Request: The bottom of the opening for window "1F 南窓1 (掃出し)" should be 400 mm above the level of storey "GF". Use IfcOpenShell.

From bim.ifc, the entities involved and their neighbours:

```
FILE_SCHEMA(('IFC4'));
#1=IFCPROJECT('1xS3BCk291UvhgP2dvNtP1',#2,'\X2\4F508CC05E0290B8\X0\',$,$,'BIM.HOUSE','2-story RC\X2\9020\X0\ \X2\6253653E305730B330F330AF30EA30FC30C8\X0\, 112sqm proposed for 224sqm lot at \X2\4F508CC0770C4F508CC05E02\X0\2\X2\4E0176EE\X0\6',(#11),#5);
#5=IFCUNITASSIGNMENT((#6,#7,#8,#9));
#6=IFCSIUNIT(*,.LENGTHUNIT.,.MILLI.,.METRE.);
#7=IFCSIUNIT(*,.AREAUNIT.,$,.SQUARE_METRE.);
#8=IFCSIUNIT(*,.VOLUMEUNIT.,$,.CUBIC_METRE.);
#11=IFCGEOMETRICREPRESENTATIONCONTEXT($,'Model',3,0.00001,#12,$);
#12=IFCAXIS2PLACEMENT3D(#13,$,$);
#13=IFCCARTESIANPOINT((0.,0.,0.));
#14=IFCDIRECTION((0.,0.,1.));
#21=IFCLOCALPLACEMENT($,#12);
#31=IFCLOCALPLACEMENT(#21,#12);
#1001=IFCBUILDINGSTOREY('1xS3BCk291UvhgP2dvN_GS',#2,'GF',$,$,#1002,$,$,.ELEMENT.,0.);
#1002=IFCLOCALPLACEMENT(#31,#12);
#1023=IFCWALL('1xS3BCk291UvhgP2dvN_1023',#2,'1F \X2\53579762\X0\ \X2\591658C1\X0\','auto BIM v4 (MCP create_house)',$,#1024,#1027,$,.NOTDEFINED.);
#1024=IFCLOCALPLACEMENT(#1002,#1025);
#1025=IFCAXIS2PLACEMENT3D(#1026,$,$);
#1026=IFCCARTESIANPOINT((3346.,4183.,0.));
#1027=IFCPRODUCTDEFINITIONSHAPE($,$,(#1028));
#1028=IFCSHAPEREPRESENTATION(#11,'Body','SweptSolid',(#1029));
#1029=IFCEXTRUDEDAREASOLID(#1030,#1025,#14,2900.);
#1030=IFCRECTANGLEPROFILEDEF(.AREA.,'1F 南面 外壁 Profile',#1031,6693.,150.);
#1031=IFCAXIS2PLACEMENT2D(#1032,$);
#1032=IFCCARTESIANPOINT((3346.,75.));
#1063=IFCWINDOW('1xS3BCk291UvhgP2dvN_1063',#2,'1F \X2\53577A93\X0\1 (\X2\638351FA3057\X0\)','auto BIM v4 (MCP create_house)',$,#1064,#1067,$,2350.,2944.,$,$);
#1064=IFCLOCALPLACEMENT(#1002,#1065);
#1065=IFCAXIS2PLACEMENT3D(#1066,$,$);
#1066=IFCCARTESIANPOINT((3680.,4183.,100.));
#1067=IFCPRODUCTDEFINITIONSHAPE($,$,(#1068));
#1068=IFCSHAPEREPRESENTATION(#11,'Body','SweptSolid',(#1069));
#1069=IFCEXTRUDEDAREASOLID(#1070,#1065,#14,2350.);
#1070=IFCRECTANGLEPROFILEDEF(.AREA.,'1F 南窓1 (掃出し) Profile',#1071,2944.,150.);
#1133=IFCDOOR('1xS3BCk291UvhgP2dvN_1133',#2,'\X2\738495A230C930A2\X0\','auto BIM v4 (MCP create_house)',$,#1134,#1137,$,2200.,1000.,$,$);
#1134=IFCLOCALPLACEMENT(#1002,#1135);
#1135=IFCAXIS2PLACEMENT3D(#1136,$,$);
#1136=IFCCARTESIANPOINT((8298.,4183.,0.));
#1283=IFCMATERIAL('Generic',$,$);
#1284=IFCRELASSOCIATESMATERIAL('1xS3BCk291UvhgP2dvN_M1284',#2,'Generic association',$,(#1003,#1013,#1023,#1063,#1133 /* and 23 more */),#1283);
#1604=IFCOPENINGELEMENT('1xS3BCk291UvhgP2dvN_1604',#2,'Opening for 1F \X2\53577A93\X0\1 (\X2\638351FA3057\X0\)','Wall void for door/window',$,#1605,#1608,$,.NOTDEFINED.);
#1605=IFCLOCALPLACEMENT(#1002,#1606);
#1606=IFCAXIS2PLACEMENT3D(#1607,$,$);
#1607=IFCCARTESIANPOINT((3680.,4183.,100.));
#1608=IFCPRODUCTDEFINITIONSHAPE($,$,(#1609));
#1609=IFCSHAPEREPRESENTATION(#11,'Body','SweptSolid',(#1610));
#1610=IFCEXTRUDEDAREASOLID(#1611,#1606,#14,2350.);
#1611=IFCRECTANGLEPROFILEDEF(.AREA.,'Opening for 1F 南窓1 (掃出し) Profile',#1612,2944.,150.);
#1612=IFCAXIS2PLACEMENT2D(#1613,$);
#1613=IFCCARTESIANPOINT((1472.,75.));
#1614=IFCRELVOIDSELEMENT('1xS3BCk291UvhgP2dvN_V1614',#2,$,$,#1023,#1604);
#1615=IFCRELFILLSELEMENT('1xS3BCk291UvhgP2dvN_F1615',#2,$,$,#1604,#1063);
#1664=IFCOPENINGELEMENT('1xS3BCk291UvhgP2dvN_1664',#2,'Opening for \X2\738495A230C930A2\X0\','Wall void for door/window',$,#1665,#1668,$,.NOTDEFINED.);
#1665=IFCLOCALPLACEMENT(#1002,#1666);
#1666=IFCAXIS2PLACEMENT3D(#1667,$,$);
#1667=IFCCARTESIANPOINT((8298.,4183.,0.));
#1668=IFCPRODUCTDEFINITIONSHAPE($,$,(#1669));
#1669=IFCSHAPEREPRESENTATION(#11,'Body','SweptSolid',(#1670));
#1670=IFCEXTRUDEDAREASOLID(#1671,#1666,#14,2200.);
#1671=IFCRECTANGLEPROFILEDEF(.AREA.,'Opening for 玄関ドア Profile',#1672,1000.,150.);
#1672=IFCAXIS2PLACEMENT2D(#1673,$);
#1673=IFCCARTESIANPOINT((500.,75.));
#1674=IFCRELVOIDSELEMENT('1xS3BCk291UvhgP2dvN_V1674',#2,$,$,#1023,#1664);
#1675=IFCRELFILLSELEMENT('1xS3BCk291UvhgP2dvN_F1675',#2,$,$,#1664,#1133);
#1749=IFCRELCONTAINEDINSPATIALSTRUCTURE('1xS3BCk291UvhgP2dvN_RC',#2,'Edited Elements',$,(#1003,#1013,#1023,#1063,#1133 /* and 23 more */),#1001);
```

```python
import numpy as np
import ifcopenshell
import ifcopenshell.api.geometry
import ifcopenshell.geom
import ifcopenshell.util.element
import ifcopenshell.util.placement
import ifcopenshell.util.shape
import ifcopenshell.util.unit

model = ifcopenshell.open("bim.ifc")
unit_scale = ifcopenshell.util.unit.calculate_unit_scale(model)

window = model.by_guid("1xS3BCk291UvhgP2dvN_1063")
opening = window.FillsVoids[0].RelatingOpeningElement
storey = ifcopenshell.util.element.get_container(window, ifc_class="IfcBuildingStorey")
level = ifcopenshell.util.placement.get_local_placement(storey.ObjectPlacement)[2, 3]

# The opening's origin need not be at the sill, so measure its lowest point.
shape = ifcopenshell.geom.create_shape(ifcopenshell.geom.settings(), opening)
bottom = ifcopenshell.util.shape.get_shape_bottom_elevation(shape, shape.geometry) / unit_scale
dz = level + 400.0 - bottom

shift = np.array([0.0, 0.0, dz])
# The window is not placed relative to its opening, so move both.
for product in (opening, window):
    matrix = ifcopenshell.util.placement.get_local_placement(product.ObjectPlacement)
    matrix[:3, 3] += shift
    ifcopenshell.api.geometry.edit_object_placement(model, product=product, matrix=matrix, is_si=False)

print(f"moved by {dz * unit_scale:+.3f} m")

model.write("bim_updated.ifc")
```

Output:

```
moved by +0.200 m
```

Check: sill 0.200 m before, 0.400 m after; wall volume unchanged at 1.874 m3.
